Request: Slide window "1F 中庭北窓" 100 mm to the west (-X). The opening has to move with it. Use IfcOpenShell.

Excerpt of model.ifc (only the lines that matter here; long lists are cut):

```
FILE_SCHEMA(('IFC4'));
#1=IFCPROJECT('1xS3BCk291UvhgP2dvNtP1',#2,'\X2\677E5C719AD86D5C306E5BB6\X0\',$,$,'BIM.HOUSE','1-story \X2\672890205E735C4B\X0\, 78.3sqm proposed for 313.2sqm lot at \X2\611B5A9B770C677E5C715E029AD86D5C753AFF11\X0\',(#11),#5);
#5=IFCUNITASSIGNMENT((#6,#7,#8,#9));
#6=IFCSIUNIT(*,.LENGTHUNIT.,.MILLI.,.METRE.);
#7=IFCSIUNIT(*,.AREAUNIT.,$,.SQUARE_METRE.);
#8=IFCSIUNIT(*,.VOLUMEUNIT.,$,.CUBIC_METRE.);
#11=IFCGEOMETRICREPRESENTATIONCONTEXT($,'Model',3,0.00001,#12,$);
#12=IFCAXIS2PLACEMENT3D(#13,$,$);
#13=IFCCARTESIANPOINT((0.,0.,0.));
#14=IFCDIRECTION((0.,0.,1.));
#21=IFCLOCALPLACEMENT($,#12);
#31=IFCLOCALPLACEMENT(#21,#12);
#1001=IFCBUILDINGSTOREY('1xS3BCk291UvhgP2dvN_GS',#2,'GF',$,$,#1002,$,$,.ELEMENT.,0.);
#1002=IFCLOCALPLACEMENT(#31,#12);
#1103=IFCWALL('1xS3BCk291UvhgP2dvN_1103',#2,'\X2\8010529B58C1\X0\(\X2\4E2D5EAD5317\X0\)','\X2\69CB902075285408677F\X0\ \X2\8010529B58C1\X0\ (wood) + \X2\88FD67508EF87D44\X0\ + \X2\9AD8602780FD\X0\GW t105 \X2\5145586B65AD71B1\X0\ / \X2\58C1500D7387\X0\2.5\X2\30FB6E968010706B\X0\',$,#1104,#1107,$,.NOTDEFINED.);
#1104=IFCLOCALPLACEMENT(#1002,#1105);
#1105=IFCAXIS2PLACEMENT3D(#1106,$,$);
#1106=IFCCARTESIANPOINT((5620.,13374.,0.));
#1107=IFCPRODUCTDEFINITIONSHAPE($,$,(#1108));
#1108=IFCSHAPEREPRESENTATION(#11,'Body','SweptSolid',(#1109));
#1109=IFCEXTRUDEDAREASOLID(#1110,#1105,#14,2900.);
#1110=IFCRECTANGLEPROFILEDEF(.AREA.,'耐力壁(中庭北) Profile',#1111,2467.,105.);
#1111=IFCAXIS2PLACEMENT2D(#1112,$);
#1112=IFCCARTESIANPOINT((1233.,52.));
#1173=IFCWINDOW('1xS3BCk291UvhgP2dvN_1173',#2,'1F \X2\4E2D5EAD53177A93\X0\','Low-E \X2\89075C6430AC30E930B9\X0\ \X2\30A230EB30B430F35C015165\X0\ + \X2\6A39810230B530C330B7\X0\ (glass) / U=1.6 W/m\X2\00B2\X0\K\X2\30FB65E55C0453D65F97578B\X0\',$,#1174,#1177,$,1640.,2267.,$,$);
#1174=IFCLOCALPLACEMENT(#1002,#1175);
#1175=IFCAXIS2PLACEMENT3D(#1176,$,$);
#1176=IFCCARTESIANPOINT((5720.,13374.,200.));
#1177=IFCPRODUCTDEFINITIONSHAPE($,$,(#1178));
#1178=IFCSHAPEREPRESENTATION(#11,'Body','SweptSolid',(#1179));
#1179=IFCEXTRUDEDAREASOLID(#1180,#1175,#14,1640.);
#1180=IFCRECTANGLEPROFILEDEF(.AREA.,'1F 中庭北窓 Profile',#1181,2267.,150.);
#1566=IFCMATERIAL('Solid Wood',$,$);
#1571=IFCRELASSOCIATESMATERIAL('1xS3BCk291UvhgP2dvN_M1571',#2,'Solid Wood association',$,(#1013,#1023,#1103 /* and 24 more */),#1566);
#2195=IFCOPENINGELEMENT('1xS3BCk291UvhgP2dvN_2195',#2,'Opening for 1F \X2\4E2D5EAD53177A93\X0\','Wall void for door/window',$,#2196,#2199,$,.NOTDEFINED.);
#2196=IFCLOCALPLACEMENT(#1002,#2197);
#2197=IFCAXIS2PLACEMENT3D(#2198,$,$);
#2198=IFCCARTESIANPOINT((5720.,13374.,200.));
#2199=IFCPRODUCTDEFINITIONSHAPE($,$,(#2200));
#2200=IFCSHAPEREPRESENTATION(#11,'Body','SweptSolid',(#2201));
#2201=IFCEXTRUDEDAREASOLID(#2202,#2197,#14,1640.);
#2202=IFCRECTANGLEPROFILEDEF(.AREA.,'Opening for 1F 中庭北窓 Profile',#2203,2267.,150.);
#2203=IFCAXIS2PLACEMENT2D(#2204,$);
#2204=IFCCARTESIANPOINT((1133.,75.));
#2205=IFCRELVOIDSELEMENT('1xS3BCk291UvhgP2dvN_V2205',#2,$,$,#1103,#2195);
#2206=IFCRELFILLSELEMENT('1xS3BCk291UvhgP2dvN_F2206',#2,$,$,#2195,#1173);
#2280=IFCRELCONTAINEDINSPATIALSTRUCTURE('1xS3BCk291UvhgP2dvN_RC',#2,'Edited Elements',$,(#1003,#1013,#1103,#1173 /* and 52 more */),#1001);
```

```python
import ifcopenshell
import ifcopenshell.api.geometry
import ifcopenshell.util.placement

model = ifcopenshell.open("model.ifc")

window = model.by_guid("1xS3BCk291UvhgP2dvN_1173")
opening = window.FillsVoids[0].RelatingOpeningElement
wall = opening.VoidsElements[0].RelatingBuildingElement

wall_matrix = ifcopenshell.util.placement.get_local_placement(wall.ObjectPlacement)
shift = wall_matrix[:3, 0] * -100.0
before = ifcopenshell.util.placement.get_local_placement(window.ObjectPlacement)[:3, 3].copy()

# The window is not placed relative to its opening, so move both.
for product in (opening, window):
    matrix = ifcopenshell.util.placement.get_local_placement(product.ObjectPlacement)
    matrix[:3, 3] += shift
    ifcopenshell.api.geometry.edit_object_placement(model, product=product, matrix=matrix, is_si=False)

after = ifcopenshell.util.placement.get_local_placement(window.ObjectPlacement)[:3, 3]
print("window moved by", (after - before).round(3) + 0.0)

model.write("model_edited.ifc")
```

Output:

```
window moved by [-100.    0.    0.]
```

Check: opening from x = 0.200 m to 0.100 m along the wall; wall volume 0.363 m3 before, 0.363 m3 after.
